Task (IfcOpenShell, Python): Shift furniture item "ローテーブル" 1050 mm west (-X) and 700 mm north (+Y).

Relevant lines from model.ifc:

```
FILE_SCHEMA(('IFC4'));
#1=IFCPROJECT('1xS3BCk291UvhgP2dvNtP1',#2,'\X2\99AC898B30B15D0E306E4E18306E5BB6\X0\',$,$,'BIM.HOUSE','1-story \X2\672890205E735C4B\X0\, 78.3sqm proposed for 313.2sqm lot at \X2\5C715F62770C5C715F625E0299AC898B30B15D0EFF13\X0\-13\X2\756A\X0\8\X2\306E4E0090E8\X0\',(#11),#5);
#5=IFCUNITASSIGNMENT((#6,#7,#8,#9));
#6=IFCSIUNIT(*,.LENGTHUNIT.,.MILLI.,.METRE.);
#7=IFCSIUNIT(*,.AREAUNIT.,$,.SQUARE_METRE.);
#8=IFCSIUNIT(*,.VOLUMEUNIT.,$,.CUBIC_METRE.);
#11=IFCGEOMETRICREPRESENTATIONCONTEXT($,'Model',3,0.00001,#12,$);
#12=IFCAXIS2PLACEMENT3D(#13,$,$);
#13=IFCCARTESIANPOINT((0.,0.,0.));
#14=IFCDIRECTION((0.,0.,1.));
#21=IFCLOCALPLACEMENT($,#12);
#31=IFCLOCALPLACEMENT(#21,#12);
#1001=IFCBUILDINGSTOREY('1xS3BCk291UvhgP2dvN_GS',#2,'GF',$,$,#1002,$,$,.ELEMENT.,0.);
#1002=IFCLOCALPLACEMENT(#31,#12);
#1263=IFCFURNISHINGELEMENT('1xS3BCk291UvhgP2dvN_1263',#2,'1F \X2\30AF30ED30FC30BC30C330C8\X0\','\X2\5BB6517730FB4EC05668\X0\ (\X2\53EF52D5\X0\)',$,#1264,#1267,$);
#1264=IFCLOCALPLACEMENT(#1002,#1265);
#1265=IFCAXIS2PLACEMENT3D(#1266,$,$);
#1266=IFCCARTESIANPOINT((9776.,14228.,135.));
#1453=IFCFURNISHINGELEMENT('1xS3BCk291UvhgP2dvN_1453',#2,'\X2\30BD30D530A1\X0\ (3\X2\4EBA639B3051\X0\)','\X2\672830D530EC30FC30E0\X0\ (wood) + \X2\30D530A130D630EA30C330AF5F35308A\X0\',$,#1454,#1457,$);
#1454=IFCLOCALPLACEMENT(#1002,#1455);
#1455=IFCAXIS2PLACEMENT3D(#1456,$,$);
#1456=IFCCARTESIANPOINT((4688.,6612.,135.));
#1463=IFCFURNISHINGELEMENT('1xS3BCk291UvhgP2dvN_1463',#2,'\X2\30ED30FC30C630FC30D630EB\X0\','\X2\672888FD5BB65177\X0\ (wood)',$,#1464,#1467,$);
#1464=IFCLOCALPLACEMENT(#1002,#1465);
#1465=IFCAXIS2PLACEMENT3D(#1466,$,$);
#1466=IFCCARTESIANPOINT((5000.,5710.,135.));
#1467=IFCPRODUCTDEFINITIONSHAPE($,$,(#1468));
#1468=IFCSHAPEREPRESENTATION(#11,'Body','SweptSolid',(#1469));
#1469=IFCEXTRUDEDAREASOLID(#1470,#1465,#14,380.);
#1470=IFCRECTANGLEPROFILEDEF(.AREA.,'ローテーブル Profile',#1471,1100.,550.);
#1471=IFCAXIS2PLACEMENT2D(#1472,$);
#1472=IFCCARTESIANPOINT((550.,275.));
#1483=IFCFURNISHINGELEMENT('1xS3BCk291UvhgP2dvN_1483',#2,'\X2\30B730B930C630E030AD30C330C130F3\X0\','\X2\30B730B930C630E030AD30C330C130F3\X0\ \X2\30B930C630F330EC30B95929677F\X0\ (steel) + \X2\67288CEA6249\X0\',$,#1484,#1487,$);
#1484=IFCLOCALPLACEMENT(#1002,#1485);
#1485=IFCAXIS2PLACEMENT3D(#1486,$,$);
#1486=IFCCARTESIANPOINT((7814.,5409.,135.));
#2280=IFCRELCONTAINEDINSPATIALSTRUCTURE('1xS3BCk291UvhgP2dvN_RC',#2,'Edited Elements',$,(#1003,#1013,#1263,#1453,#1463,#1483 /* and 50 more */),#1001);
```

```python
import ifcopenshell
import ifcopenshell.api.geometry
import ifcopenshell.util.placement
import ifcopenshell.util.unit

model = ifcopenshell.open("model.ifc")
unit_scale = ifcopenshell.util.unit.calculate_unit_scale(model)

item = model.by_id(1463)
matrix = ifcopenshell.util.placement.get_local_placement(item.ObjectPlacement)
matrix[0, 3] -= 1.05 / unit_scale
matrix[1, 3] += 0.7 / unit_scale
ifcopenshell.api.geometry.edit_object_placement(model, product=item, matrix=matrix, is_si=False)

print(ifcopenshell.util.placement.get_local_placement(item.ObjectPlacement).round(3) + 0.0)

model.write("model-out.ifc")
```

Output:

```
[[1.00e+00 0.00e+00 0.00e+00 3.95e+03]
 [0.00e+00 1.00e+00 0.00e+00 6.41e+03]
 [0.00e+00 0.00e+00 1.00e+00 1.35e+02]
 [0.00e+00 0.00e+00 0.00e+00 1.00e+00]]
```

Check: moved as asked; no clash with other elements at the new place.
